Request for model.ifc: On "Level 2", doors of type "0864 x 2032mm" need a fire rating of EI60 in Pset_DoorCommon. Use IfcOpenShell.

First a look at what the model holds.

```python
import ifcopenshell
import ifcopenshell.util.element

model = ifcopenshell.open("model.ifc")
print(model.schema)
storey = next(s for s in model.by_type("IfcBuildingStorey") if s.Name == "Level 2")
doors = [e for e in ifcopenshell.util.element.get_decomposition(storey) if e.is_a("IfcDoor")]
seen = {}
for e in doors:
    element_type = ifcopenshell.util.element.get_type(e)
    key = (element_type.Name if element_type != e and element_type else None, ifcopenshell.util.element.get_pset(e, "Pset_DoorCommon", "FireRating"))
    seen[key] = seen.get(key, 0) + 1
for (name, value), count in sorted(seen.items(), key=str):
    print(count, "x", name, "|", value)
```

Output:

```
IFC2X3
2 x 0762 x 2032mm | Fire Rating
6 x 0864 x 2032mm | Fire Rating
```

```python
import ifcopenshell
import ifcopenshell.api.pset
import ifcopenshell.util.element

model = ifcopenshell.open("model.ifc")

storey = next(s for s in model.by_type("IfcBuildingStorey") if s.Name == "Level 2")
doors = [e for e in ifcopenshell.util.element.get_decomposition(storey) if e.is_a("IfcDoor")]

count = 0
for e in doors:
    element_type = ifcopenshell.util.element.get_type(e)
    if element_type in (None, e) or element_type.Name != "0864 x 2032mm":
        continue
    # add_pset returns the element's existing set when there is one.
    pset = ifcopenshell.api.pset.add_pset(model, product=e, name="Pset_DoorCommon")
    ifcopenshell.api.pset.edit_pset(model, pset=pset, properties={"FireRating": "EI60"})
    count += 1

print(count, "doors updated")

model.write("model_v2.ifc")
```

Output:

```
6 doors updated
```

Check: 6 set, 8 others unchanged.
